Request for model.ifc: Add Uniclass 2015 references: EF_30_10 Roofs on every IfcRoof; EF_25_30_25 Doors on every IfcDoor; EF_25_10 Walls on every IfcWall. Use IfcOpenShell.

First a look at what the model holds.

```python
import ifcopenshell

model = ifcopenshell.open("model.ifc")
print(model.schema)
print("classifications:", [c.Name for c in model.by_type("IfcClassification")])
for ifc_class in ("IfcDoor", "IfcRoof", "IfcStair", "IfcWall", "IfcWindow"):
    print(ifc_class, len(model.by_type(ifc_class)))
```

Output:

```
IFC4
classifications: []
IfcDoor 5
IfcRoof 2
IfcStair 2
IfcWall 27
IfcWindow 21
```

```python
import ifcopenshell
import ifcopenshell.api.classification

model = ifcopenshell.open("model.ifc")

system = ifcopenshell.api.classification.add_classification(model, classification="Uniclass 2015")

codes = {
    "IfcRoof": ("EF_30_10", "Roofs"),
    "IfcDoor": ("EF_25_30_25", "Doors"),
    "IfcWall": ("EF_25_10", "Walls"),
}
for ifc_class, (code, name) in codes.items():
    products = model.by_type(ifc_class)
    ifcopenshell.api.classification.add_reference(
        model, products=products, classification=system, identification=code, name=name
    )
    print(code, len(products))

model.write("model_v2.ifc")
```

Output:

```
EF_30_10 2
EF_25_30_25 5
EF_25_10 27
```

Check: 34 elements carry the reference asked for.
